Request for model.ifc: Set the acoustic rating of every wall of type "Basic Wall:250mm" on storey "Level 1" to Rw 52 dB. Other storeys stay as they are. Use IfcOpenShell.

First a look at what the model holds.

```python
import ifcopenshell
import ifcopenshell.util.element

model = ifcopenshell.open("model.ifc")
print(model.schema)
storey = next(s for s in model.by_type("IfcBuildingStorey") if s.Name == "Level 1")
walls = [e for e in ifcopenshell.util.element.get_decomposition(storey) if e.is_a("IfcWall")]
seen = {}
for e in walls:
    element_type = ifcopenshell.util.element.get_type(e)
    key = (element_type.Name if element_type != e and element_type else None, ifcopenshell.util.element.get_pset(e, "Pset_WallCommon", "AcousticRating"))
    seen[key] = seen.get(key, 0) + 1
for (name, value), count in sorted(seen.items(), key=str):
    print(count, "x", name, "|", value)
```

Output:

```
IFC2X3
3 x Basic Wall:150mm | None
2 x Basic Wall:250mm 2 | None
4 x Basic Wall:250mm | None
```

```python
import ifcopenshell
import ifcopenshell.api.pset
import ifcopenshell.util.element

model = ifcopenshell.open("model.ifc")

storey = next(s for s in model.by_type("IfcBuildingStorey") if s.Name == "Level 1")
walls = [e for e in ifcopenshell.util.element.get_decomposition(storey) if e.is_a("IfcWall")]

count = 0
for e in walls:
    element_type = ifcopenshell.util.element.get_type(e)
    if element_type in (None, e) or element_type.Name != "Basic Wall:250mm":
        continue
    # add_pset returns the element's existing set when there is one.
    pset = ifcopenshell.api.pset.add_pset(model, product=e, name="Pset_WallCommon")
    ifcopenshell.api.pset.edit_pset(model, pset=pset, properties={"AcousticRating": "Rw 52 dB"})
    count += 1

print(count, "walls updated")

model.write("model_rev.ifc")
```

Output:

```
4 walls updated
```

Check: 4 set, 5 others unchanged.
